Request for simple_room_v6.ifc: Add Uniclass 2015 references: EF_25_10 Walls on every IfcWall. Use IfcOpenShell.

First a look at what the model holds.

```python
import ifcopenshell

model = ifcopenshell.open("simple_room_v6.ifc")
print(model.schema)
print("classifications:", [c.Name for c in model.by_type("IfcClassification")])
for ifc_class in ("IfcDoor", "IfcRoof", "IfcStair", "IfcWall", "IfcWindow"):
    print(ifc_class, len(model.by_type(ifc_class)))
```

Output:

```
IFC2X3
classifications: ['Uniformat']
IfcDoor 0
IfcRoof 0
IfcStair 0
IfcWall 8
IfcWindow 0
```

```python
import ifcopenshell
import ifcopenshell.api.classification

model = ifcopenshell.open("simple_room_v6.ifc")

# IFC2X3 requires Source and Edition and has no link from the project to the system.
system = model.create_entity("IfcClassification", Source="NBS", Edition="2015", Name="Uniclass 2015")

codes = {
    "IfcWall": ("EF_25_10", "Walls"),
}
for ifc_class, (code, name) in codes.items():
    products = model.by_type(ifc_class)
    ifcopenshell.api.classification.add_reference(
        model, products=products, classification=system, identification=code, name=name
    )
    print(code, len(products))

model.write("simple_room_v6_v2.ifc")
```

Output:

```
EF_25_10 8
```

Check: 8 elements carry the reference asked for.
